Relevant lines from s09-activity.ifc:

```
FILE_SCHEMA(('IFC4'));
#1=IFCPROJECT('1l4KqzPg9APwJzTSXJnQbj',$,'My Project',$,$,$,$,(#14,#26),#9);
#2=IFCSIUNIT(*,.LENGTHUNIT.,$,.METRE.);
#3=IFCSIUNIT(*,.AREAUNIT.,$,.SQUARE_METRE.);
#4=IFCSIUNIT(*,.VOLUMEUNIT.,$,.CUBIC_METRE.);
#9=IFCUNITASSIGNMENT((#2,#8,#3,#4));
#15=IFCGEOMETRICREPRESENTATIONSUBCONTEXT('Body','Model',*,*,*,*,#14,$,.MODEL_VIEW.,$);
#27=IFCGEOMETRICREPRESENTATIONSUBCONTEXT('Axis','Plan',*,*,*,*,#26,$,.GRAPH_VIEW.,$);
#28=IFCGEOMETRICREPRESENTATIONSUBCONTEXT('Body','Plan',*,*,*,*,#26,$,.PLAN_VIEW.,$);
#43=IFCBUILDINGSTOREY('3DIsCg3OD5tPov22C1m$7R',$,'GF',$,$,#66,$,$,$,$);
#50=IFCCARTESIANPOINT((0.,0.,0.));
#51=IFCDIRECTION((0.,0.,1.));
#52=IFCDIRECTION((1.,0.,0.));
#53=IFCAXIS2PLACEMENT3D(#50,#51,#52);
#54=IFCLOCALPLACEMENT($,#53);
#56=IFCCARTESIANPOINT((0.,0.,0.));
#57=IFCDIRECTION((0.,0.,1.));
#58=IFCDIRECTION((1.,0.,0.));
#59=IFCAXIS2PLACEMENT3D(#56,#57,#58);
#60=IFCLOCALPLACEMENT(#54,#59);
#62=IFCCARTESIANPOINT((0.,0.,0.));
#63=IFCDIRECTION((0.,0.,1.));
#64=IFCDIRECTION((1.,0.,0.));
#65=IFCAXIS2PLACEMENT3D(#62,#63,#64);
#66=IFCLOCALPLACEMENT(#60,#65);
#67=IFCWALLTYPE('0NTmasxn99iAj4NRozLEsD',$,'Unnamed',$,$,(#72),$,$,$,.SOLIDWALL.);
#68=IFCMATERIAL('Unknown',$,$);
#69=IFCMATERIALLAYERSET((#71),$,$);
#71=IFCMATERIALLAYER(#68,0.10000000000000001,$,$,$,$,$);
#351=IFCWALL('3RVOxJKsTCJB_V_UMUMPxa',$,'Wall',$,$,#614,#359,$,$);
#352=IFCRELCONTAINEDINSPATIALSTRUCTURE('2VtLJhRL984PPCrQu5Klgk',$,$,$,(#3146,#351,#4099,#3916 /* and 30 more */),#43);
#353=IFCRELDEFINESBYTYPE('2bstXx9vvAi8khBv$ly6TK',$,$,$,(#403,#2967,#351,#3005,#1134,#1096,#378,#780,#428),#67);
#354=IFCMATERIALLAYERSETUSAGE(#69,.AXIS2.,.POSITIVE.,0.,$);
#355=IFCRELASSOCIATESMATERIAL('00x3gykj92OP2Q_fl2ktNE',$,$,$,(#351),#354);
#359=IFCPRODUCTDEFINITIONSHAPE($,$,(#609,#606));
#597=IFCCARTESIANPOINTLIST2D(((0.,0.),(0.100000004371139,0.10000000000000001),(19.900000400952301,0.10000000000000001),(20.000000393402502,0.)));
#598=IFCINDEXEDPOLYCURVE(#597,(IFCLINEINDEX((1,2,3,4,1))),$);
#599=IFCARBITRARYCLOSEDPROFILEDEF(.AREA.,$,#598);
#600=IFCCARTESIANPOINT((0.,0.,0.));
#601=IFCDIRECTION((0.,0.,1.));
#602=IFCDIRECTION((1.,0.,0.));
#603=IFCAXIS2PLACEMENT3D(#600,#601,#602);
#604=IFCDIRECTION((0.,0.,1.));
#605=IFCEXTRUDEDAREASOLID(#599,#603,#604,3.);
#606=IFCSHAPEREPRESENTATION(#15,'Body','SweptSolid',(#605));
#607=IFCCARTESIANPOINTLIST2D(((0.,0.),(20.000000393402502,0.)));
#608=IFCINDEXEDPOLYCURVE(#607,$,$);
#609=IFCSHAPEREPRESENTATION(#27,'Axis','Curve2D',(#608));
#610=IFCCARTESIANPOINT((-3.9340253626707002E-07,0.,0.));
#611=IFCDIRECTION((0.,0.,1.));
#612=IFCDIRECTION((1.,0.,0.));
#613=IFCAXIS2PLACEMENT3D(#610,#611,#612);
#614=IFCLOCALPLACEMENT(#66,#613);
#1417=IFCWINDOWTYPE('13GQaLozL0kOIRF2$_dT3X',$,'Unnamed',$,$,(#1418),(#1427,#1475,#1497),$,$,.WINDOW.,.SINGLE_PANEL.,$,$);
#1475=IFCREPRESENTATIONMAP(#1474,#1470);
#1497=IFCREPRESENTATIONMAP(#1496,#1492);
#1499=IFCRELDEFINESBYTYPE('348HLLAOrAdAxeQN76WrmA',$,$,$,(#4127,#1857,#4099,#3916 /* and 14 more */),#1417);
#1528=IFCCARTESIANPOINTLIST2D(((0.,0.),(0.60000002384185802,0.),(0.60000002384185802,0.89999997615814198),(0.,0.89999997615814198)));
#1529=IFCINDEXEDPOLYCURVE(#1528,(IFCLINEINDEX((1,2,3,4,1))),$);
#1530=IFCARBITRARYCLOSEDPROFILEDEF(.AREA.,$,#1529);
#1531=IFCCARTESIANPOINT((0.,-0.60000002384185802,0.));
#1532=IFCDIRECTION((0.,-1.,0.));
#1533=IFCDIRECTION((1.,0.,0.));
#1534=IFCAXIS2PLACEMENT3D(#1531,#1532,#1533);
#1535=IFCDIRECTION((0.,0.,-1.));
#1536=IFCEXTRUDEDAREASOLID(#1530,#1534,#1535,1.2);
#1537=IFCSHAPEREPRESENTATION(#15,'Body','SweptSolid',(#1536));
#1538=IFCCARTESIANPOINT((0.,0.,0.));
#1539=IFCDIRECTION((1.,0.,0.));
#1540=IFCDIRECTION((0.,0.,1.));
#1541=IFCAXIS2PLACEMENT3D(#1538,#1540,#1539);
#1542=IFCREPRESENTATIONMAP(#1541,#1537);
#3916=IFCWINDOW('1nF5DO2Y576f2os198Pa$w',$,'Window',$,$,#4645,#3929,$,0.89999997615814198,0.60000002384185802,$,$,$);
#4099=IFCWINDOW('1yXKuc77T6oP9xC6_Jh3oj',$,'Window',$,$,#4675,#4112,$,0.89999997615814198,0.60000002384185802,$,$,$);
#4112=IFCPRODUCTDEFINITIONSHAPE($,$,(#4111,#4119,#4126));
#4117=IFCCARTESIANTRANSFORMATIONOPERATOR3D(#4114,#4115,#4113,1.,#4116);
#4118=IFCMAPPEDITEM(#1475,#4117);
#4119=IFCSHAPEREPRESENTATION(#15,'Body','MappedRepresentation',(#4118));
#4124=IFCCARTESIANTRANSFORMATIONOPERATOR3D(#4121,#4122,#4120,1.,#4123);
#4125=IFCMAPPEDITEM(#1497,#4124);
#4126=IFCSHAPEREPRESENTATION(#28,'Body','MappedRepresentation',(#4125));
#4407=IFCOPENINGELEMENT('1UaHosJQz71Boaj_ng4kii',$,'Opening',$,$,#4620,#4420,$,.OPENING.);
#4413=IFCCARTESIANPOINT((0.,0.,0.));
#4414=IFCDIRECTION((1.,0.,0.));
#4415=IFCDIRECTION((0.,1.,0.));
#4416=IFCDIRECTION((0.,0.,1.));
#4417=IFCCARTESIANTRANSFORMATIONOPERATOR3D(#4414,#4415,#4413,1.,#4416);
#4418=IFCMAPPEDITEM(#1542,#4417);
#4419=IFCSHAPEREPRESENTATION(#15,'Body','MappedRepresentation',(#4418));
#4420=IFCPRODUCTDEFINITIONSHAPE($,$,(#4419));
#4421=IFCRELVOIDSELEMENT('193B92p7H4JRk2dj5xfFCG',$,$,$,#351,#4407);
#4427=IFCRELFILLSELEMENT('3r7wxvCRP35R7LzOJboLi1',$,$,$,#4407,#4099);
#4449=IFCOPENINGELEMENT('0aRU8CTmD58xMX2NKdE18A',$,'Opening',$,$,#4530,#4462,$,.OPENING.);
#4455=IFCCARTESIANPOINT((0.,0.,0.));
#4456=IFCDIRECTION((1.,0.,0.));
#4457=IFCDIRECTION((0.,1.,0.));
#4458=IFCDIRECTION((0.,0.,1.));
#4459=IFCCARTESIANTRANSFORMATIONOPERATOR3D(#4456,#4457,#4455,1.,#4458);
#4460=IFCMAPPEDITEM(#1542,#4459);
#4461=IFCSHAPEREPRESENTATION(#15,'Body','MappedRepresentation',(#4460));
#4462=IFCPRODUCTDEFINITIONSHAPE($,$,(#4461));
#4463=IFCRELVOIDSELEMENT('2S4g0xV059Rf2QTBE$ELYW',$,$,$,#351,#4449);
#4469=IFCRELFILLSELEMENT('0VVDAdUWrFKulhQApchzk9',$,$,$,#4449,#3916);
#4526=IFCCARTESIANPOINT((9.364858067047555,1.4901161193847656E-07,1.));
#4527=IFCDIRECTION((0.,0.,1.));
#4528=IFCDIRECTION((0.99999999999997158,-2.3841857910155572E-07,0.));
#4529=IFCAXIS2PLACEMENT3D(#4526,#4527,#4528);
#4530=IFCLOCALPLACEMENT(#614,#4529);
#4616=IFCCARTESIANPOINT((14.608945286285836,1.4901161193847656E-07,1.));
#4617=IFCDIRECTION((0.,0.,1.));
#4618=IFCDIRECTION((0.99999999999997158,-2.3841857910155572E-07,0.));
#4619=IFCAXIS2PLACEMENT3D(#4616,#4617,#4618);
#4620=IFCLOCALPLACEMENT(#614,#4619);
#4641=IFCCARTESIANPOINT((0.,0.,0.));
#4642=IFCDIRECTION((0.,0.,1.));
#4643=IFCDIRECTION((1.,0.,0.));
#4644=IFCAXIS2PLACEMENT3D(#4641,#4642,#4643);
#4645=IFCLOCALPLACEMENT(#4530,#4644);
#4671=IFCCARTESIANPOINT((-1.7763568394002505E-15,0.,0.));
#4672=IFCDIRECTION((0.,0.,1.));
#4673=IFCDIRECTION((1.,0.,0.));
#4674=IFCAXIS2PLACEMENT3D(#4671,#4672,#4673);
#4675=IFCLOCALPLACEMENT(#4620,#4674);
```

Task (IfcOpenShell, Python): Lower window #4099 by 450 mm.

```python
import numpy as np
import ifcopenshell
import ifcopenshell.api.geometry
import ifcopenshell.util.placement
import ifcopenshell.util.unit

model = ifcopenshell.open("s09-activity.ifc")
unit_scale = ifcopenshell.util.unit.calculate_unit_scale(model)

window = model.by_guid("1yXKuc77T6oP9xC6_Jh3oj")
opening = window.FillsVoids[0].RelatingOpeningElement
dz = -0.45 / unit_scale

shift = np.array([0.0, 0.0, dz])
# The window is placed relative to its opening, so it follows when the opening moves.
matrix = ifcopenshell.util.placement.get_local_placement(opening.ObjectPlacement)
matrix[:3, 3] += shift
ifcopenshell.api.geometry.edit_object_placement(
    model, product=opening, matrix=matrix, is_si=False, should_transform_children=True
)

print(f"moved by {dz * unit_scale:+.3f} m")

model.write("s09-activity_updated.ifc")
```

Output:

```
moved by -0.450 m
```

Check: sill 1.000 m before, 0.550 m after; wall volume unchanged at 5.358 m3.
